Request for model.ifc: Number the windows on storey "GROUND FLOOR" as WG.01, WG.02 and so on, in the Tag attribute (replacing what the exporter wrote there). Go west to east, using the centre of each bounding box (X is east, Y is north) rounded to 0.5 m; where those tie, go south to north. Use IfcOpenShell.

First a look at what the model holds.

```python
import ifcopenshell
import ifcopenshell.util.element
import ifcopenshell.util.placement

model = ifcopenshell.open("model.ifc")
print(model.schema)
storey = next(s for s in model.by_type("IfcBuildingStorey") if s.Name == "GROUND FLOOR")
windows = [e for e in ifcopenshell.util.element.get_decomposition(storey) if e.is_a("IfcWindow")]
for e in sorted(windows, key=lambda e: e.id()):
    origin = ifcopenshell.util.placement.get_local_placement(e.ObjectPlacement)[:3, 3]
    print(e.id(), e.Tag, e.Name, origin.round(2) + 0.0, sep=" | ")
```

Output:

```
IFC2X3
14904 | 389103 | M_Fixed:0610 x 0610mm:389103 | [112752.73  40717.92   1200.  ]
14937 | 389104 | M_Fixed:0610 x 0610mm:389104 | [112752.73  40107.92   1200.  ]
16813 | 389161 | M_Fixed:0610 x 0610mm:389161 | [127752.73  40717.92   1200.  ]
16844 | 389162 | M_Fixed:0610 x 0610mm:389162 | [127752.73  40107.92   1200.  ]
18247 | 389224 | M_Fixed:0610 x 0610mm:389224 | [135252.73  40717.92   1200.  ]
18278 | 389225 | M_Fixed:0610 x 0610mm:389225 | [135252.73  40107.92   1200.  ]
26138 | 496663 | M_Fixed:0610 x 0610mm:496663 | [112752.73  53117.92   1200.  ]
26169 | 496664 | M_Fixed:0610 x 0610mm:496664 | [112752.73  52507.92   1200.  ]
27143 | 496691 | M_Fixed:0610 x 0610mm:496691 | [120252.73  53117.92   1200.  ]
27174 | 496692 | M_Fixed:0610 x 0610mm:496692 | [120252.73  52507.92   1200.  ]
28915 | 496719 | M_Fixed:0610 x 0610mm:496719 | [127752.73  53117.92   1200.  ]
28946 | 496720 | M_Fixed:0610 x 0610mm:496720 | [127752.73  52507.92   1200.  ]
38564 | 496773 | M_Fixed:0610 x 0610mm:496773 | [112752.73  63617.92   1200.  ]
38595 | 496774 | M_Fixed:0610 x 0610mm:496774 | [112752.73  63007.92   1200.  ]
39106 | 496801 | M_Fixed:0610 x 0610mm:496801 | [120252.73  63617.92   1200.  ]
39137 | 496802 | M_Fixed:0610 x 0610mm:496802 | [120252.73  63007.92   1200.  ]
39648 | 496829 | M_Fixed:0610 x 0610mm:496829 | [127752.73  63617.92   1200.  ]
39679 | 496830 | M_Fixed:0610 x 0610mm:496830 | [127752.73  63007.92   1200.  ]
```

```python
import ifcopenshell
import ifcopenshell.geom
import ifcopenshell.util.element
import ifcopenshell.util.shape

model = ifcopenshell.open("model.ifc")
settings = ifcopenshell.geom.settings()
settings.set("use-world-coords", True)


def centre(element):
    shape = ifcopenshell.geom.create_shape(settings, element)
    return ifcopenshell.util.shape.get_bbox_centroid(shape.geometry)


storey = next(s for s in model.by_type("IfcBuildingStorey") if s.Name == "GROUND FLOOR")
windows = [e for e in ifcopenshell.util.element.get_decomposition(storey) if e.is_a("IfcWindow")]

# Insertion points can sit at a corner or the storey origin, so sort by the geometry (in metres).
centres = {e: centre(e) for e in windows}
windows.sort(key=lambda e: (round(centres[e][0] / 0.5), centres[e][1]))

for i, e in enumerate(windows, start=1):
    number = f"WG.{i:02d}"
    e.Tag = number
    print(e.id(), number)

model.write("model_rev.ifc")
```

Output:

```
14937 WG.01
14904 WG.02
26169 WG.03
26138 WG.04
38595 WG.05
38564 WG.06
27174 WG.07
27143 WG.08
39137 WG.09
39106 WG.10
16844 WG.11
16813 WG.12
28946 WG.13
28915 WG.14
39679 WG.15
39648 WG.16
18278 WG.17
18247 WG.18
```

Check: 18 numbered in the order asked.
